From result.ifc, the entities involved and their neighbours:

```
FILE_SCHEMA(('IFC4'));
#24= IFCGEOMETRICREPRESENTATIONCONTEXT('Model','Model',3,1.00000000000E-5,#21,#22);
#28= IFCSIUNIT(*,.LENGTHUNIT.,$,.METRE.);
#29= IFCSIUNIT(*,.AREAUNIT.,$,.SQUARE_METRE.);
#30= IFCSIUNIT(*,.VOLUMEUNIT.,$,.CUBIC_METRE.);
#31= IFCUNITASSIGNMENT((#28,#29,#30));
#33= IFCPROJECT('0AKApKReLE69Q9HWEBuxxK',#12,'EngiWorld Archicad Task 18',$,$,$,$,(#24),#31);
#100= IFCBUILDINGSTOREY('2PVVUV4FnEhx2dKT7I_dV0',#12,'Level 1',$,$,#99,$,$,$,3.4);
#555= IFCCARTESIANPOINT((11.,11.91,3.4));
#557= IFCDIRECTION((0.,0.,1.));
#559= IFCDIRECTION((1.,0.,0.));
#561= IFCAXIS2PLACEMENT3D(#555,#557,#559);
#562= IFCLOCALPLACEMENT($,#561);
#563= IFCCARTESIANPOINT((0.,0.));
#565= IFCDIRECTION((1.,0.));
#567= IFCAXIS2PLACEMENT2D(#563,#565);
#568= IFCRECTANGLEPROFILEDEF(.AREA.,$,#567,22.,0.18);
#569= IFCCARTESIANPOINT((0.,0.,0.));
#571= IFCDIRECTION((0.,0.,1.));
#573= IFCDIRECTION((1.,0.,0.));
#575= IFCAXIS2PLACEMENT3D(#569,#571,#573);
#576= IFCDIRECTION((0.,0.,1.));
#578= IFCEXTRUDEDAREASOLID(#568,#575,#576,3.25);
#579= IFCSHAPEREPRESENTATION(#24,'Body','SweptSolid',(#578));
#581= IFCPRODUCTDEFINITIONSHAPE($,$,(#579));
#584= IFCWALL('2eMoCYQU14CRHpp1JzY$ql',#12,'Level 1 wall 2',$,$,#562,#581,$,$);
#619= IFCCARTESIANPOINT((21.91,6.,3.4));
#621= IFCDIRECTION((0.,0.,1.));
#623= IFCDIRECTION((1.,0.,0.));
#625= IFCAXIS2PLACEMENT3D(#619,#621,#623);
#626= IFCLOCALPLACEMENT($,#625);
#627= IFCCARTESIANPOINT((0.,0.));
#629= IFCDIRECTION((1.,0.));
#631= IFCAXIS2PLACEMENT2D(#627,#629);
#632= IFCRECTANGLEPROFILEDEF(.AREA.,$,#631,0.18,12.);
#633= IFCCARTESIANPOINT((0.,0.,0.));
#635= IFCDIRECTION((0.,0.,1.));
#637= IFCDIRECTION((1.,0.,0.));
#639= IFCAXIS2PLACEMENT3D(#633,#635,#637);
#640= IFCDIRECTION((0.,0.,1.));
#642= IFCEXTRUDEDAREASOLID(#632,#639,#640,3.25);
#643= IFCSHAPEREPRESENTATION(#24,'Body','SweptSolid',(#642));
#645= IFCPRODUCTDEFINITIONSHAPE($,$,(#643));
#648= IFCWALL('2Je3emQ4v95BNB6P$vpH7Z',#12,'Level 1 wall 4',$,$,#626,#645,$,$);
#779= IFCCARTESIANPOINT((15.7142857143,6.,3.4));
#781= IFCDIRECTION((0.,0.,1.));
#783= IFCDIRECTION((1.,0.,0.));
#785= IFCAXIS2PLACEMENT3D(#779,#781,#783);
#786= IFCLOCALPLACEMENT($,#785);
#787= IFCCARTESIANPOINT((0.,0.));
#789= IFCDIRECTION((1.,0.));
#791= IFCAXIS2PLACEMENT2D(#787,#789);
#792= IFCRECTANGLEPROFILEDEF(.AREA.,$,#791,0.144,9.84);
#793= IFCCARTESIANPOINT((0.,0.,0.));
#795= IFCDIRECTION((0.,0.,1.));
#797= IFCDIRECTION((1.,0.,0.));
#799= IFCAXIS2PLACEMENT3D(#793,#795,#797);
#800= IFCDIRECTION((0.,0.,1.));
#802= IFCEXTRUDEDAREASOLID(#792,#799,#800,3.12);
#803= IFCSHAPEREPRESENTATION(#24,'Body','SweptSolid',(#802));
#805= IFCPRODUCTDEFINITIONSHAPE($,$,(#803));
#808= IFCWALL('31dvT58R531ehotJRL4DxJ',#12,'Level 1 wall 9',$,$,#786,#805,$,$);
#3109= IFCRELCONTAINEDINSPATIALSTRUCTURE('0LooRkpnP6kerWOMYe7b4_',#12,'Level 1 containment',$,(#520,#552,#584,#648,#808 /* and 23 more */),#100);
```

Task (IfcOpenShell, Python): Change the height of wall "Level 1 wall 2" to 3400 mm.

```python
import ifcopenshell
import ifcopenshell.geom
import ifcopenshell.util.shape

model = ifcopenshell.open("result.ifc")
settings = ifcopenshell.geom.settings()


def volume(element):
    """Net volume in cubic metres, openings subtracted."""
    shape = ifcopenshell.geom.create_shape(settings, element)
    return ifcopenshell.util.shape.get_volume(shape.geometry)


wall = model.by_guid("2eMoCYQU14CRHpp1JzY$ql")
before = volume(wall)

body = next(r for r in wall.Representation.Representations if r.RepresentationIdentifier == "Body")
solid = body.Items[0]
old_height = solid.Depth
solid.Depth = 3.4
after = volume(wall)

print(f"height {old_height:g} -> {solid.Depth:g}, volume {before:.3f} -> {after:.3f} m3")

model.write("result_updated.ifc")
```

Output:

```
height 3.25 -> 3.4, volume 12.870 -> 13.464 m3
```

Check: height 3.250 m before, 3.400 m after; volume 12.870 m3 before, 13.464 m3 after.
